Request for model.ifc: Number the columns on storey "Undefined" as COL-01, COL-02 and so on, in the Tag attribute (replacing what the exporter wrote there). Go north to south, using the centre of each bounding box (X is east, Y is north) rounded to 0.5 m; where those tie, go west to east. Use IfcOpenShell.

First a look at what the model holds.

```python
import ifcopenshell
import ifcopenshell.util.element
import ifcopenshell.util.placement

model = ifcopenshell.open("model.ifc")
print(model.schema)
storey = next(s for s in model.by_type("IfcBuildingStorey") if s.Name == "Undefined")
columns = [e for e in ifcopenshell.util.element.get_decomposition(storey) if e.is_a("IfcColumn")]
for e in sorted(columns, key=lambda e: e.id()):
    origin = ifcopenshell.util.placement.get_local_placement(e.ObjectPlacement)[:3, 3]
    print(e.id(), e.Tag, e.Name, origin.round(2) + 0.0, sep=" | ")
```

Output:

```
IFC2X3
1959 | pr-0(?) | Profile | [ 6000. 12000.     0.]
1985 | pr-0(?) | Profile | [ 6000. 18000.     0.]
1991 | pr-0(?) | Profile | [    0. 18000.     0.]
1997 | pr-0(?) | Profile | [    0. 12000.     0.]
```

```python
import ifcopenshell
import ifcopenshell.geom
import ifcopenshell.util.element
import ifcopenshell.util.shape

model = ifcopenshell.open("model.ifc")
settings = ifcopenshell.geom.settings()
settings.set("use-world-coords", True)


def centre(element):
    shape = ifcopenshell.geom.create_shape(settings, element)
    return ifcopenshell.util.shape.get_bbox_centroid(shape.geometry)


storey = next(s for s in model.by_type("IfcBuildingStorey") if s.Name == "Undefined")
columns = [e for e in ifcopenshell.util.element.get_decomposition(storey) if e.is_a("IfcColumn")]

# Insertion points can sit at a corner or the storey origin, so sort by the geometry (in metres).
centres = {e: centre(e) for e in columns}
columns.sort(key=lambda e: (-round(centres[e][1] / 0.5), centres[e][0]))

for i, e in enumerate(columns, start=1):
    number = f"COL-{i:02d}"
    e.Tag = number
    print(e.id(), number)

model.write("model_edited.ifc")
```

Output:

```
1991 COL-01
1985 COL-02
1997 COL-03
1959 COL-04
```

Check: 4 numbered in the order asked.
